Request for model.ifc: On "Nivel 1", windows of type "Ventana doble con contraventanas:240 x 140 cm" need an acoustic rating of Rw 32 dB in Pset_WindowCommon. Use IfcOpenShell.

First a look at what the model holds.

```python
import ifcopenshell
import ifcopenshell.util.element

model = ifcopenshell.open("model.ifc")
print(model.schema)
storey = next(s for s in model.by_type("IfcBuildingStorey") if s.Name == "Nivel 1")
windows = [e for e in ifcopenshell.util.element.get_decomposition(storey) if e.is_a("IfcWindow")]
seen = {}
for e in windows:
    element_type = ifcopenshell.util.element.get_type(e)
    key = (element_type.Name if element_type != e and element_type else None, ifcopenshell.util.element.get_pset(e, "Pset_WindowCommon", "AcousticRating"))
    seen[key] = seen.get(key, 0) + 1
for (name, value), count in sorted(seen.items(), key=str):
    print(count, "x", name, "|", value)
```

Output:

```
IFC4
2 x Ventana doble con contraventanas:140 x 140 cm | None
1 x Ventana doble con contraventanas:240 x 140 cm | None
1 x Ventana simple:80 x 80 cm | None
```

```python
import ifcopenshell
import ifcopenshell.api.pset
import ifcopenshell.util.element

model = ifcopenshell.open("model.ifc")

storey = next(s for s in model.by_type("IfcBuildingStorey") if s.Name == "Nivel 1")
windows = [e for e in ifcopenshell.util.element.get_decomposition(storey) if e.is_a("IfcWindow")]

count = 0
for e in windows:
    element_type = ifcopenshell.util.element.get_type(e)
    if element_type in (None, e) or element_type.Name != "Ventana doble con contraventanas:240 x 140 cm":
        continue
    # add_pset returns the element's existing set when there is one.
    pset = ifcopenshell.api.pset.add_pset(model, product=e, name="Pset_WindowCommon")
    ifcopenshell.api.pset.edit_pset(model, pset=pset, properties={"AcousticRating": "Rw 32 dB"})
    count += 1

print(count, "windows updated")

model.write("model_v2.ifc")
```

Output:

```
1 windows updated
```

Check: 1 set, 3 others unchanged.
